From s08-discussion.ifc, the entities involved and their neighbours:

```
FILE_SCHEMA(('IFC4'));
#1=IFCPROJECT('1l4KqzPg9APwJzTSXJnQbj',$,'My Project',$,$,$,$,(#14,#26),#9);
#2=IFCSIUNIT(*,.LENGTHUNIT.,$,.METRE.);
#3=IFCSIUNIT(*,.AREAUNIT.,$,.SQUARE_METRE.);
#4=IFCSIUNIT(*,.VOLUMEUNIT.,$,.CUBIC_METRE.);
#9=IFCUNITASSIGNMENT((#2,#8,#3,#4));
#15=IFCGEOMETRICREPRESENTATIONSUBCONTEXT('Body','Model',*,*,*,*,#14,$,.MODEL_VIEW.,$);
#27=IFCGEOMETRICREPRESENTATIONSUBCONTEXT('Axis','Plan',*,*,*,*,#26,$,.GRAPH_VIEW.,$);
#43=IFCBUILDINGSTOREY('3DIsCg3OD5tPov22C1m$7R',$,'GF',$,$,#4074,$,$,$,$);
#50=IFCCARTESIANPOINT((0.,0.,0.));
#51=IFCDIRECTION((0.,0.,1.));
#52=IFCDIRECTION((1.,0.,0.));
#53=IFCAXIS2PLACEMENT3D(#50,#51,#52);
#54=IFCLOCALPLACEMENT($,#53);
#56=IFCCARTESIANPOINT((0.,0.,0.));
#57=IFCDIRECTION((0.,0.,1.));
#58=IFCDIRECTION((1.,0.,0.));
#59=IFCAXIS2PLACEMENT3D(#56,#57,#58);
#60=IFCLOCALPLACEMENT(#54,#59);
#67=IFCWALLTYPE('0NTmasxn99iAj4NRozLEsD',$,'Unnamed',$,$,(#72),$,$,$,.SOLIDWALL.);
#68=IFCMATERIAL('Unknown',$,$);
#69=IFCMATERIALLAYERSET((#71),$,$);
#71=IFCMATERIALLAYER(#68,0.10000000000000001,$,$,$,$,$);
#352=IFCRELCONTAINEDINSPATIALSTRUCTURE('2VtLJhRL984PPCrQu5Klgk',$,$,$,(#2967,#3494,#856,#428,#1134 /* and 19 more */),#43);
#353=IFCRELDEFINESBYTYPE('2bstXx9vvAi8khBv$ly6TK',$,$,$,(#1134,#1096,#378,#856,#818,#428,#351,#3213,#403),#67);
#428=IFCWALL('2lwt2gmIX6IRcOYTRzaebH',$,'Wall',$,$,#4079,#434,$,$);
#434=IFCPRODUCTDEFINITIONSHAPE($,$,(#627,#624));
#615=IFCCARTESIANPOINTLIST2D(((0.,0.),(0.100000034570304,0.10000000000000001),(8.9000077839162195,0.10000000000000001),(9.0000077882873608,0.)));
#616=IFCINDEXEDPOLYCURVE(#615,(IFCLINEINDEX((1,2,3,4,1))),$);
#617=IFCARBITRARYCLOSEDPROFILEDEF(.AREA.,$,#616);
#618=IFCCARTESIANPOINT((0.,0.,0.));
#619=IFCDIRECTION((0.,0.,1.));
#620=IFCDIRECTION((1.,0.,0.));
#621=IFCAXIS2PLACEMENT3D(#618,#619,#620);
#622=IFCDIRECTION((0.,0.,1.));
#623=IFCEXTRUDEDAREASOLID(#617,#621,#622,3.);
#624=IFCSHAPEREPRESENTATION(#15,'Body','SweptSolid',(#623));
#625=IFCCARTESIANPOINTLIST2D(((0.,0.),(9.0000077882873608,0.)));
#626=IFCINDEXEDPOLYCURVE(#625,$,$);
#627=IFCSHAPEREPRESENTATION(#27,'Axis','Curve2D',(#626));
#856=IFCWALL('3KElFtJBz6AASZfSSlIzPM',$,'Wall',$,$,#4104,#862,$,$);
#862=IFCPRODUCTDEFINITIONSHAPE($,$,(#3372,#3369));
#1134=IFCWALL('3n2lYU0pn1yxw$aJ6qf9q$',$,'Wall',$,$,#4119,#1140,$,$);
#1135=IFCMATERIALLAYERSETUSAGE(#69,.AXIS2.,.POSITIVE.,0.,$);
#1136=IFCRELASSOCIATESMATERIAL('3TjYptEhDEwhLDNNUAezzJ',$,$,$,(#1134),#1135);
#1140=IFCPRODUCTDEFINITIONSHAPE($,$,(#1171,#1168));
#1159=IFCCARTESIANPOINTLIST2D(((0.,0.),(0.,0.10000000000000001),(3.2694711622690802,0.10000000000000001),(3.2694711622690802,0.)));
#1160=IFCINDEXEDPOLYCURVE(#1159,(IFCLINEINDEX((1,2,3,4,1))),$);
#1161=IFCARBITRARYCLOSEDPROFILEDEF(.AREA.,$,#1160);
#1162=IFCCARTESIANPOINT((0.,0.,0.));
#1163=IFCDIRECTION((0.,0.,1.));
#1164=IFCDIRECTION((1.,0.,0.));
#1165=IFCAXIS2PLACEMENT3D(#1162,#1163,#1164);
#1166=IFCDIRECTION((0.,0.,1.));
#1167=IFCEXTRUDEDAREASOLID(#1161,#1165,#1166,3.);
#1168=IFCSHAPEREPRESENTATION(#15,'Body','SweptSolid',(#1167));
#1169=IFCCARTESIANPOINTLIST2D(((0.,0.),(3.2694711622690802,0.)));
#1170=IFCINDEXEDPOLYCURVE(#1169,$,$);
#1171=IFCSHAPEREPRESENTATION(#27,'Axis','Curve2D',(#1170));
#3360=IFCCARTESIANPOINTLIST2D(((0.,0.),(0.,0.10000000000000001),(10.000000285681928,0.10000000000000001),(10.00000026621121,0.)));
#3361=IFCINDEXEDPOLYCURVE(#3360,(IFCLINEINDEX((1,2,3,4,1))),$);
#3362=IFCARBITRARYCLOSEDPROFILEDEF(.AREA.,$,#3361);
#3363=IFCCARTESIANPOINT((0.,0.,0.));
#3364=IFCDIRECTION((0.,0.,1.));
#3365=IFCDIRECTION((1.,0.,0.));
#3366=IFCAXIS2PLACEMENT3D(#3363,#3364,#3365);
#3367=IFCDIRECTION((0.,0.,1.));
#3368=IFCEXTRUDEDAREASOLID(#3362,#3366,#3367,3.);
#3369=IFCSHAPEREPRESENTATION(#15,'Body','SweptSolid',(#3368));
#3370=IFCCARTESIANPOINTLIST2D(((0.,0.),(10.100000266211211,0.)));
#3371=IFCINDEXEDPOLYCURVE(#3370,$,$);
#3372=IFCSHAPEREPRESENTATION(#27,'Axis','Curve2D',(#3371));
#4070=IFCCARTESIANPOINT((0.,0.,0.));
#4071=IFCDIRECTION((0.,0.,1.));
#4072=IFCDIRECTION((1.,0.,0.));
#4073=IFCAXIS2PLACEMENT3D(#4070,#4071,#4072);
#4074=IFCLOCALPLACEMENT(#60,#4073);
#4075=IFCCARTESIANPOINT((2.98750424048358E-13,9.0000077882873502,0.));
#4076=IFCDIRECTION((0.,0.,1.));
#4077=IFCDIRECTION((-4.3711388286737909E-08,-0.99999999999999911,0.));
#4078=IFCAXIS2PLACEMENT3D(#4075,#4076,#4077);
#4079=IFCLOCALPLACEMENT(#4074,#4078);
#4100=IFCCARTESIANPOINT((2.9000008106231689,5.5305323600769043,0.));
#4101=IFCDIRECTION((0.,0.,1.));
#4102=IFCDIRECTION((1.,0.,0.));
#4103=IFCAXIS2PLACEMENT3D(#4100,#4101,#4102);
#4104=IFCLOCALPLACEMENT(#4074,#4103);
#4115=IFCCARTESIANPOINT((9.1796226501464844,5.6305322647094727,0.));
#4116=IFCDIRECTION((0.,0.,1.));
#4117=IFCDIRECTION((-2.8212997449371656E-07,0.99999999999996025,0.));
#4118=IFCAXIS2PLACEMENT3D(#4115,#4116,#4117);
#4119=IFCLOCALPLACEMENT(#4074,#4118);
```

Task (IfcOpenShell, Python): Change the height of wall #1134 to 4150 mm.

```python
import ifcopenshell
import ifcopenshell.geom
import ifcopenshell.util.representation
import ifcopenshell.util.shape
import ifcopenshell.util.unit

model = ifcopenshell.open("s08-discussion.ifc")
unit_scale = ifcopenshell.util.unit.calculate_unit_scale(model)
settings = ifcopenshell.geom.settings()


def volume(element):
    """Net volume in cubic metres, openings subtracted."""
    shape = ifcopenshell.geom.create_shape(settings, element)
    return ifcopenshell.util.shape.get_volume(shape.geometry)


wall = model.by_guid("3n2lYU0pn1yxw$aJ6qf9q$")
before = volume(wall)

body = ifcopenshell.util.representation.get_representation(wall, "Model", "Body")
solid = body.Items[0]
old_height = solid.Depth
solid.Depth = 4.15 / unit_scale
after = volume(wall)

print(f"height {old_height:g} -> {solid.Depth:g}, volume {before:.3f} -> {after:.3f} m3")

model.write("s08-discussion_updated.ifc")
```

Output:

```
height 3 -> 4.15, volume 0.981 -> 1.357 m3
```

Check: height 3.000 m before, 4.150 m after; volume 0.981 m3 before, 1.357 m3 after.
